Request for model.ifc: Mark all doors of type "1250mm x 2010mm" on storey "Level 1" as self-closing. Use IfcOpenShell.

First a look at what the model holds.

```python
import ifcopenshell
import ifcopenshell.util.element

model = ifcopenshell.open("model.ifc")
print(model.schema)
storey = next(s for s in model.by_type("IfcBuildingStorey") if s.Name == "Level 1")
doors = [e for e in ifcopenshell.util.element.get_decomposition(storey) if e.is_a("IfcDoor")]
seen = {}
for e in doors:
    element_type = ifcopenshell.util.element.get_type(e)
    key = (element_type.Name if element_type != e and element_type else None, ifcopenshell.util.element.get_pset(e, "Pset_DoorCommon", "SelfClosing"))
    seen[key] = seen.get(key, 0) + 1
for (name, value), count in sorted(seen.items(), key=str):
    print(count, "x", name, "|", value)
```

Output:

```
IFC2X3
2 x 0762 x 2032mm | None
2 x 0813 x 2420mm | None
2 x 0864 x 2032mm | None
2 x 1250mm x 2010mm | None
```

```python
import ifcopenshell
import ifcopenshell.api.pset
import ifcopenshell.util.element

model = ifcopenshell.open("model.ifc")

storey = next(s for s in model.by_type("IfcBuildingStorey") if s.Name == "Level 1")
doors = [e for e in ifcopenshell.util.element.get_decomposition(storey) if e.is_a("IfcDoor")]

count = 0
for e in doors:
    element_type = ifcopenshell.util.element.get_type(e)
    if element_type in (None, e) or element_type.Name != "1250mm x 2010mm":
        continue
    # add_pset returns the element's existing set when there is one.
    pset = ifcopenshell.api.pset.add_pset(model, product=e, name="Pset_DoorCommon")
    ifcopenshell.api.pset.edit_pset(model, pset=pset, properties={"SelfClosing": True})
    count += 1

print(count, "doors updated")

model.write("model_updated.ifc")
```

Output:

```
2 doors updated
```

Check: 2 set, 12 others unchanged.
